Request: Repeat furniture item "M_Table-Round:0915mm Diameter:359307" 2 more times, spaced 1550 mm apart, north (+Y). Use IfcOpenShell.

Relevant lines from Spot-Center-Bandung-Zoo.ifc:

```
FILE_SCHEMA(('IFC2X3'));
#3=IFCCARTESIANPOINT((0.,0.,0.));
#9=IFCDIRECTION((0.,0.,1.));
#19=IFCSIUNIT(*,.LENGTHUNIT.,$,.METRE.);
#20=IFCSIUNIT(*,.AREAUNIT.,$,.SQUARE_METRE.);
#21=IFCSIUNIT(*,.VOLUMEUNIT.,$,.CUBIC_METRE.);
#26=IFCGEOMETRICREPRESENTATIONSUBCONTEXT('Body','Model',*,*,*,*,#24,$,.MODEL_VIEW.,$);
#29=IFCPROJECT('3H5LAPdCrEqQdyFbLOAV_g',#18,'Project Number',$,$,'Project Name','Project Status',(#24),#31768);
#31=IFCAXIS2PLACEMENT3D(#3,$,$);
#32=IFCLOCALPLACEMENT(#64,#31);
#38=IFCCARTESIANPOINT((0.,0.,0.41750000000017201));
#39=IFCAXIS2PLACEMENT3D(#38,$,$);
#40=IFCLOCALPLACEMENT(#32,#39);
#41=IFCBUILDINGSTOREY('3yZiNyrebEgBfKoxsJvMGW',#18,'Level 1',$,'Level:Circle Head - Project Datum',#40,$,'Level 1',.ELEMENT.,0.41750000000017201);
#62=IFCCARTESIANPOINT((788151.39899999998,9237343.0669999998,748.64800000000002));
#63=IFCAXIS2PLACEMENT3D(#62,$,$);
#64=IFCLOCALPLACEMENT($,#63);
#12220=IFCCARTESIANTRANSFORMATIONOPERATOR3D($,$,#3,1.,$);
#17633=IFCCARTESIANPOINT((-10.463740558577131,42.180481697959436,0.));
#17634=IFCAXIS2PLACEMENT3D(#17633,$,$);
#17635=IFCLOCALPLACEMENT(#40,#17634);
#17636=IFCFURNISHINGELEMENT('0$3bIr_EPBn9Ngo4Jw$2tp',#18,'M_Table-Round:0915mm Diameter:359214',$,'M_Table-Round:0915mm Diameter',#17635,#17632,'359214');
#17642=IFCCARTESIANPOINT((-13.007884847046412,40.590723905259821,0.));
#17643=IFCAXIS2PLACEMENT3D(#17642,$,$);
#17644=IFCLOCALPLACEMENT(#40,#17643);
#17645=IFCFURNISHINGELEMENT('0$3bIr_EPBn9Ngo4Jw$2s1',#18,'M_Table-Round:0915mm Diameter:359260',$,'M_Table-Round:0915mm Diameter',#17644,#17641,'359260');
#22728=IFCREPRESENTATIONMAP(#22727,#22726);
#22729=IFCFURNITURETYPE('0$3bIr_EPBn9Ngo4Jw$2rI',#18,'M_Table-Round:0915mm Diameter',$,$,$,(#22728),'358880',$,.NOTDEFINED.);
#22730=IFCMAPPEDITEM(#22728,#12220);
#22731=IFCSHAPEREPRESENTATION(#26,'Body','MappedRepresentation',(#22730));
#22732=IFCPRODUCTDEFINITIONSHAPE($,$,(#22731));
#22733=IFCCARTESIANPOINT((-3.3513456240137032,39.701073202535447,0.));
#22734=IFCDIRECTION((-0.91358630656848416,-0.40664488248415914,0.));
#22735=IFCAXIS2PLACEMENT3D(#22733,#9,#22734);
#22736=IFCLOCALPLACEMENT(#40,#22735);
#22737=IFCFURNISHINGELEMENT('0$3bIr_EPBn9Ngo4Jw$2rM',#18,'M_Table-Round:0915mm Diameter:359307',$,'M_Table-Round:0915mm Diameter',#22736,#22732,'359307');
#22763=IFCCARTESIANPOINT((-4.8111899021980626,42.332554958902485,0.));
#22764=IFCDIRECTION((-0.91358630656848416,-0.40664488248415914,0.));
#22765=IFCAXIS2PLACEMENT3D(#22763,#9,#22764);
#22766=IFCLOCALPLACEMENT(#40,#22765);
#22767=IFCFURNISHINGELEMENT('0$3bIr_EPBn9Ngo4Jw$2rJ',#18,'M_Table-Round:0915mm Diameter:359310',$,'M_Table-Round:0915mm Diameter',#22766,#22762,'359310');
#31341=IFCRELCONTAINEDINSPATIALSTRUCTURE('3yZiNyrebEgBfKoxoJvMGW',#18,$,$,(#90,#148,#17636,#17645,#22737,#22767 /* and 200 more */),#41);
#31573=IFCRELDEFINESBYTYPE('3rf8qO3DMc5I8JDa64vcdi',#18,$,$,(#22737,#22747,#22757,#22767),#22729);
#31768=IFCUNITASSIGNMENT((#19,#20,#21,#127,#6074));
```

```python
import numpy as np
import ifcopenshell
import ifcopenshell.api.geometry
import ifcopenshell.api.root
import ifcopenshell.util.element
import ifcopenshell.util.placement

model = ifcopenshell.open("Spot-Center-Bandung-Zoo.ifc")


def reuse_history(source, copy):
    """copy_class also copies each property set's owner history, people and application; keep the originals."""
    for rel in copy.IsDefinedBy:
        if rel.is_a("IfcRelDefinesByProperties") and (history := rel.RelatingPropertyDefinition.OwnerHistory):
            rel.RelatingPropertyDefinition.OwnerHistory = source.OwnerHistory
            ifcopenshell.util.element.remove_deep2(model, history)


source = model.by_id(22737)
base = ifcopenshell.util.placement.get_local_placement(source.ObjectPlacement)
step = np.array([0.0, 1.0, 0.0]) * 1.55

for i in range(1, 3):
    copy = ifcopenshell.api.root.copy_class(model, product=source)
    copy.Representation = ifcopenshell.util.element.copy_deep(
        model, source.Representation, exclude=["IfcGeometricRepresentationContext", "IfcRepresentationMap"]
    )
    copy.Name = "M_Table-Round:0915mm Diameter"
    copy.Tag = None
    reuse_history(source, copy)
    matrix = base.copy()
    matrix[:3, 3] += i * step
    print("added at", matrix[:3, 3].round(3) + 0.0)
    ifcopenshell.api.geometry.edit_object_placement(model, product=copy, matrix=matrix, is_si=False)

model.write("Spot-Center-Bandung-Zoo_updated.ifc")
```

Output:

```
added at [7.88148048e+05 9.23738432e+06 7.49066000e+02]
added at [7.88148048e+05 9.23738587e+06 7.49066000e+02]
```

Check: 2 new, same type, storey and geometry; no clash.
